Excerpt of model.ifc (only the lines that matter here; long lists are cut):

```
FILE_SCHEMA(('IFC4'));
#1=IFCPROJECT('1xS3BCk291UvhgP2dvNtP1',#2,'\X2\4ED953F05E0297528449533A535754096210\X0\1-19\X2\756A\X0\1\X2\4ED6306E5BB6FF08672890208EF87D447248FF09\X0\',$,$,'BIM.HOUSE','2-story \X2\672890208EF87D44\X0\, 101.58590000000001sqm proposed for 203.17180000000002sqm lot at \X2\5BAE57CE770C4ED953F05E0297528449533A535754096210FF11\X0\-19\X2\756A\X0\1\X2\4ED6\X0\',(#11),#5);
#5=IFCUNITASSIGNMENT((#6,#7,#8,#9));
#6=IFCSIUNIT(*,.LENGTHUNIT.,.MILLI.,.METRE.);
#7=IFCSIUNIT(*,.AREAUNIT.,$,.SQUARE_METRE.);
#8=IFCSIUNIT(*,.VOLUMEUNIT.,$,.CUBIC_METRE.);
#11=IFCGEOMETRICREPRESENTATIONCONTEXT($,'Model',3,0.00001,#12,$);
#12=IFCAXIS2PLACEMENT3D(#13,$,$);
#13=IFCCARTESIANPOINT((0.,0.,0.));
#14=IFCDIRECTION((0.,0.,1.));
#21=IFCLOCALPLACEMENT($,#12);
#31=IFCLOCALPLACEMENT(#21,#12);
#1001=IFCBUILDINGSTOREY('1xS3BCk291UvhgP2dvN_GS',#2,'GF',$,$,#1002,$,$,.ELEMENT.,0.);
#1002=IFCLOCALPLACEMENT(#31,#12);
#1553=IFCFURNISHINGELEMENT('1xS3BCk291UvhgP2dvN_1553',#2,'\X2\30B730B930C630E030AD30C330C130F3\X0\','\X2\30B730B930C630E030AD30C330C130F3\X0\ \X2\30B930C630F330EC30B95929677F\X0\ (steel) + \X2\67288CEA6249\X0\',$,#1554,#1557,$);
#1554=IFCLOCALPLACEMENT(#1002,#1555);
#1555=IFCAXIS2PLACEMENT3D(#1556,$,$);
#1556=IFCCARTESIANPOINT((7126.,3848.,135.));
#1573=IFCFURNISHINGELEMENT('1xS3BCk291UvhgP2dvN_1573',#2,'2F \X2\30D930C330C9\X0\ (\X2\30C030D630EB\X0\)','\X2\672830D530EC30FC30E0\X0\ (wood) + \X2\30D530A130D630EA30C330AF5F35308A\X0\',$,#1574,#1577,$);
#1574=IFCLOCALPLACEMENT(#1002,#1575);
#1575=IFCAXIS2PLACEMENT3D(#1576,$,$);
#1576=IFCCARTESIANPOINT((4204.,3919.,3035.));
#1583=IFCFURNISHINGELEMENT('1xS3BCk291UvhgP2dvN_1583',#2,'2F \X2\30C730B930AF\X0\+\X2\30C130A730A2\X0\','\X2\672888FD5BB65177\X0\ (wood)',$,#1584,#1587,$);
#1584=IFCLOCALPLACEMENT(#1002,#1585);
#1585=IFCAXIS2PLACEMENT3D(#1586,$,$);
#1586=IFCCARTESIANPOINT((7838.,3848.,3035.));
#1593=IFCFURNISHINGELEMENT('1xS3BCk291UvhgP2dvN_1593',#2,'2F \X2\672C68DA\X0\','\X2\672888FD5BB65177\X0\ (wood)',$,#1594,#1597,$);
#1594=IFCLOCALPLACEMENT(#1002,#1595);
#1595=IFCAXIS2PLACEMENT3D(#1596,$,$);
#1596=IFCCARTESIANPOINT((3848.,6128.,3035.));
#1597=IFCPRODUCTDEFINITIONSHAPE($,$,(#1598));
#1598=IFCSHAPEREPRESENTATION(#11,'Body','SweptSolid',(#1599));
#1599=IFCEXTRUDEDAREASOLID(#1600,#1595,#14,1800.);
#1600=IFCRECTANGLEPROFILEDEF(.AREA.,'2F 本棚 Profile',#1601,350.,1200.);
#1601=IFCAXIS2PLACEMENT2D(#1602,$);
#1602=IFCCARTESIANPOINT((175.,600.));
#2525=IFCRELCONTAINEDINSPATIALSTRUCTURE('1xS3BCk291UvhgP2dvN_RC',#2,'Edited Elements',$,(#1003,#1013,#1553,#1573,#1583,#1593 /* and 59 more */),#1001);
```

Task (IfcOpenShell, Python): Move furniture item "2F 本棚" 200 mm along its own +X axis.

```python
import ifcopenshell
import ifcopenshell.api.geometry
import ifcopenshell.util.placement
import ifcopenshell.util.unit

model = ifcopenshell.open("model.ifc")
unit_scale = ifcopenshell.util.unit.calculate_unit_scale(model)

item = model.by_guid("1xS3BCk291UvhgP2dvN_1593")
matrix = ifcopenshell.util.placement.get_local_placement(item.ObjectPlacement)
matrix[:3, 3] += matrix[:3, 0] * 0.2 / unit_scale
ifcopenshell.api.geometry.edit_object_placement(model, product=item, matrix=matrix, is_si=False)

print(ifcopenshell.util.placement.get_local_placement(item.ObjectPlacement).round(3) + 0.0)

model.write("model_rev.ifc")
```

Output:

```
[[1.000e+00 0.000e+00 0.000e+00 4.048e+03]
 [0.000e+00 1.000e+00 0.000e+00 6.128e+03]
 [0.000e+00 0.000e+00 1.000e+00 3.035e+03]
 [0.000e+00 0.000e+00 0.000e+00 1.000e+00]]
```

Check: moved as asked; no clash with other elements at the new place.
